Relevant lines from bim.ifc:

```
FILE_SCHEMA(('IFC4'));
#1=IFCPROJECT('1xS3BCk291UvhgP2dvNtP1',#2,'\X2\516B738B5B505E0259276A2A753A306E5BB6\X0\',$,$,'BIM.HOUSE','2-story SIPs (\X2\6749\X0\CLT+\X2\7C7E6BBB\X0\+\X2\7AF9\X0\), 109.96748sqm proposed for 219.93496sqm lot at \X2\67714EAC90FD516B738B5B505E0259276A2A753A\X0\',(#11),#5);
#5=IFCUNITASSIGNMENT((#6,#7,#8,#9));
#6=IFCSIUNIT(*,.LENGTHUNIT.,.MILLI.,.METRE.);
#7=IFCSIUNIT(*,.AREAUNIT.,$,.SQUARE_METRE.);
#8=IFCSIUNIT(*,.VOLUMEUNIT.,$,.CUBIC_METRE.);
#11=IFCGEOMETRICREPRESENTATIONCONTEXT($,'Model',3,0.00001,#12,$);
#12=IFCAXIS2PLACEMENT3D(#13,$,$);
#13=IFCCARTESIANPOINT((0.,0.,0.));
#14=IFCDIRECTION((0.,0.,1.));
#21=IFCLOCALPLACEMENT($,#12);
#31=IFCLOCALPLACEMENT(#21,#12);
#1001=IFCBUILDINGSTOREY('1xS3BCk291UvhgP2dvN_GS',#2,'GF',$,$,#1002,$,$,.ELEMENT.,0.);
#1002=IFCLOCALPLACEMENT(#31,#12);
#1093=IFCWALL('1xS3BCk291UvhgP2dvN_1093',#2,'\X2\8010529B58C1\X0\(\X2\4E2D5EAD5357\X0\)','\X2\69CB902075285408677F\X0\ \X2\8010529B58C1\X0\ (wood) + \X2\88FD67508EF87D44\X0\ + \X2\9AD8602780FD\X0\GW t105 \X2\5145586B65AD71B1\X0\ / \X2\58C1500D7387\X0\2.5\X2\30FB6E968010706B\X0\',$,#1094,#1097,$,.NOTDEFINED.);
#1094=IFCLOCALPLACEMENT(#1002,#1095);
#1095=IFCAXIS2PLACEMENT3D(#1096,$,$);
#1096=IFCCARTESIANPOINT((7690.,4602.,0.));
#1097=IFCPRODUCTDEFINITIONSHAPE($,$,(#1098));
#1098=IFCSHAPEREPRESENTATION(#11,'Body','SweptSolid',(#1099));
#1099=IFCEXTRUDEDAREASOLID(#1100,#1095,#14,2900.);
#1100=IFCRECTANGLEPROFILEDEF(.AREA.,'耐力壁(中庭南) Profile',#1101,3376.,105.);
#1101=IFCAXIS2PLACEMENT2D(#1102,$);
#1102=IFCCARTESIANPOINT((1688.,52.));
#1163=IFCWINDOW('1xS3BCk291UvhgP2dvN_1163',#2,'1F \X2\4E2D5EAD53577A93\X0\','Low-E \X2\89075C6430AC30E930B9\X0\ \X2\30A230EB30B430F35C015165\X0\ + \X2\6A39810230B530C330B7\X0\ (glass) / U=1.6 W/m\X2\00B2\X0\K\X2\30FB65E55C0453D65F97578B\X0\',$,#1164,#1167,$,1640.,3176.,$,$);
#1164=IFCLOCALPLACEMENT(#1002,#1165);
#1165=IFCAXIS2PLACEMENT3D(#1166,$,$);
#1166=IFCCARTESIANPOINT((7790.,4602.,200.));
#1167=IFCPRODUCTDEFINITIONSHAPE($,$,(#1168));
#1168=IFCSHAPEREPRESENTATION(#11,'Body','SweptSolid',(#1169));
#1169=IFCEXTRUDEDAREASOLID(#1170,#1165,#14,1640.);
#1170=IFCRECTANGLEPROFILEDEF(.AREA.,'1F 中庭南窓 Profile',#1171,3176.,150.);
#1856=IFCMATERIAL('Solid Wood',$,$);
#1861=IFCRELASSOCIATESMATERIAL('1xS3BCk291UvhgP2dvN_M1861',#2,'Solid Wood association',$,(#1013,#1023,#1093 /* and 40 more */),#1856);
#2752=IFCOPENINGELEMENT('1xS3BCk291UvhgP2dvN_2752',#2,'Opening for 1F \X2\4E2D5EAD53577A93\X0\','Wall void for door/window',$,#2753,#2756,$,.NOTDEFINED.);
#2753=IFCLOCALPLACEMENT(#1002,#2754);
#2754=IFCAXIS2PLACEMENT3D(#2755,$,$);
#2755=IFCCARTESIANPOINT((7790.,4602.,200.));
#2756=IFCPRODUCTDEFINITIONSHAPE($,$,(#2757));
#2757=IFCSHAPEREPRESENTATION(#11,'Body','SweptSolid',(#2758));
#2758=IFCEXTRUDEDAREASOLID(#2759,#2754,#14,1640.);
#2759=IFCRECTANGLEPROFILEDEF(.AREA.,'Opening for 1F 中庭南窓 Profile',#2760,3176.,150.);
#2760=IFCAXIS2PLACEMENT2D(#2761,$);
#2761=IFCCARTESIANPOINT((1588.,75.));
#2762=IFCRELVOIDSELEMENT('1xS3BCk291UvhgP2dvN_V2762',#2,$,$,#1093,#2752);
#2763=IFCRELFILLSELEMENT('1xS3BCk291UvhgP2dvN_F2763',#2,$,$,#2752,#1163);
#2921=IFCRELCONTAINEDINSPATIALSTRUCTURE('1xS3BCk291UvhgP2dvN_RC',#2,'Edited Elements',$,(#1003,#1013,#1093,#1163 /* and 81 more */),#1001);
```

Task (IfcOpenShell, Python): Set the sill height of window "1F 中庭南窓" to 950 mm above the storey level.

```python
import numpy as np
import ifcopenshell
import ifcopenshell.api.geometry
import ifcopenshell.geom
import ifcopenshell.util.element
import ifcopenshell.util.placement
import ifcopenshell.util.shape
import ifcopenshell.util.unit

model = ifcopenshell.open("bim.ifc")
unit_scale = ifcopenshell.util.unit.calculate_unit_scale(model)

window = model.by_guid("1xS3BCk291UvhgP2dvN_1163")
opening = window.FillsVoids[0].RelatingOpeningElement
storey = ifcopenshell.util.element.get_container(window, ifc_class="IfcBuildingStorey")
level = ifcopenshell.util.placement.get_local_placement(storey.ObjectPlacement)[2, 3]

# The opening's origin need not be at the sill, so measure its lowest point.
shape = ifcopenshell.geom.create_shape(ifcopenshell.geom.settings(), opening)
bottom = ifcopenshell.util.shape.get_shape_bottom_elevation(shape, shape.geometry) / unit_scale
dz = level + 0.95 / unit_scale - bottom

shift = np.array([0.0, 0.0, dz])
# The window is not placed relative to its opening, so move both.
for product in (opening, window):
    matrix = ifcopenshell.util.placement.get_local_placement(product.ObjectPlacement)
    matrix[:3, 3] += shift
    ifcopenshell.api.geometry.edit_object_placement(model, product=product, matrix=matrix, is_si=False)

print(f"moved by {dz * unit_scale:+.3f} m")

model.write("bim_rev.ifc")
```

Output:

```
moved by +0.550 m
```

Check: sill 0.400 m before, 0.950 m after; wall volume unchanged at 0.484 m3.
